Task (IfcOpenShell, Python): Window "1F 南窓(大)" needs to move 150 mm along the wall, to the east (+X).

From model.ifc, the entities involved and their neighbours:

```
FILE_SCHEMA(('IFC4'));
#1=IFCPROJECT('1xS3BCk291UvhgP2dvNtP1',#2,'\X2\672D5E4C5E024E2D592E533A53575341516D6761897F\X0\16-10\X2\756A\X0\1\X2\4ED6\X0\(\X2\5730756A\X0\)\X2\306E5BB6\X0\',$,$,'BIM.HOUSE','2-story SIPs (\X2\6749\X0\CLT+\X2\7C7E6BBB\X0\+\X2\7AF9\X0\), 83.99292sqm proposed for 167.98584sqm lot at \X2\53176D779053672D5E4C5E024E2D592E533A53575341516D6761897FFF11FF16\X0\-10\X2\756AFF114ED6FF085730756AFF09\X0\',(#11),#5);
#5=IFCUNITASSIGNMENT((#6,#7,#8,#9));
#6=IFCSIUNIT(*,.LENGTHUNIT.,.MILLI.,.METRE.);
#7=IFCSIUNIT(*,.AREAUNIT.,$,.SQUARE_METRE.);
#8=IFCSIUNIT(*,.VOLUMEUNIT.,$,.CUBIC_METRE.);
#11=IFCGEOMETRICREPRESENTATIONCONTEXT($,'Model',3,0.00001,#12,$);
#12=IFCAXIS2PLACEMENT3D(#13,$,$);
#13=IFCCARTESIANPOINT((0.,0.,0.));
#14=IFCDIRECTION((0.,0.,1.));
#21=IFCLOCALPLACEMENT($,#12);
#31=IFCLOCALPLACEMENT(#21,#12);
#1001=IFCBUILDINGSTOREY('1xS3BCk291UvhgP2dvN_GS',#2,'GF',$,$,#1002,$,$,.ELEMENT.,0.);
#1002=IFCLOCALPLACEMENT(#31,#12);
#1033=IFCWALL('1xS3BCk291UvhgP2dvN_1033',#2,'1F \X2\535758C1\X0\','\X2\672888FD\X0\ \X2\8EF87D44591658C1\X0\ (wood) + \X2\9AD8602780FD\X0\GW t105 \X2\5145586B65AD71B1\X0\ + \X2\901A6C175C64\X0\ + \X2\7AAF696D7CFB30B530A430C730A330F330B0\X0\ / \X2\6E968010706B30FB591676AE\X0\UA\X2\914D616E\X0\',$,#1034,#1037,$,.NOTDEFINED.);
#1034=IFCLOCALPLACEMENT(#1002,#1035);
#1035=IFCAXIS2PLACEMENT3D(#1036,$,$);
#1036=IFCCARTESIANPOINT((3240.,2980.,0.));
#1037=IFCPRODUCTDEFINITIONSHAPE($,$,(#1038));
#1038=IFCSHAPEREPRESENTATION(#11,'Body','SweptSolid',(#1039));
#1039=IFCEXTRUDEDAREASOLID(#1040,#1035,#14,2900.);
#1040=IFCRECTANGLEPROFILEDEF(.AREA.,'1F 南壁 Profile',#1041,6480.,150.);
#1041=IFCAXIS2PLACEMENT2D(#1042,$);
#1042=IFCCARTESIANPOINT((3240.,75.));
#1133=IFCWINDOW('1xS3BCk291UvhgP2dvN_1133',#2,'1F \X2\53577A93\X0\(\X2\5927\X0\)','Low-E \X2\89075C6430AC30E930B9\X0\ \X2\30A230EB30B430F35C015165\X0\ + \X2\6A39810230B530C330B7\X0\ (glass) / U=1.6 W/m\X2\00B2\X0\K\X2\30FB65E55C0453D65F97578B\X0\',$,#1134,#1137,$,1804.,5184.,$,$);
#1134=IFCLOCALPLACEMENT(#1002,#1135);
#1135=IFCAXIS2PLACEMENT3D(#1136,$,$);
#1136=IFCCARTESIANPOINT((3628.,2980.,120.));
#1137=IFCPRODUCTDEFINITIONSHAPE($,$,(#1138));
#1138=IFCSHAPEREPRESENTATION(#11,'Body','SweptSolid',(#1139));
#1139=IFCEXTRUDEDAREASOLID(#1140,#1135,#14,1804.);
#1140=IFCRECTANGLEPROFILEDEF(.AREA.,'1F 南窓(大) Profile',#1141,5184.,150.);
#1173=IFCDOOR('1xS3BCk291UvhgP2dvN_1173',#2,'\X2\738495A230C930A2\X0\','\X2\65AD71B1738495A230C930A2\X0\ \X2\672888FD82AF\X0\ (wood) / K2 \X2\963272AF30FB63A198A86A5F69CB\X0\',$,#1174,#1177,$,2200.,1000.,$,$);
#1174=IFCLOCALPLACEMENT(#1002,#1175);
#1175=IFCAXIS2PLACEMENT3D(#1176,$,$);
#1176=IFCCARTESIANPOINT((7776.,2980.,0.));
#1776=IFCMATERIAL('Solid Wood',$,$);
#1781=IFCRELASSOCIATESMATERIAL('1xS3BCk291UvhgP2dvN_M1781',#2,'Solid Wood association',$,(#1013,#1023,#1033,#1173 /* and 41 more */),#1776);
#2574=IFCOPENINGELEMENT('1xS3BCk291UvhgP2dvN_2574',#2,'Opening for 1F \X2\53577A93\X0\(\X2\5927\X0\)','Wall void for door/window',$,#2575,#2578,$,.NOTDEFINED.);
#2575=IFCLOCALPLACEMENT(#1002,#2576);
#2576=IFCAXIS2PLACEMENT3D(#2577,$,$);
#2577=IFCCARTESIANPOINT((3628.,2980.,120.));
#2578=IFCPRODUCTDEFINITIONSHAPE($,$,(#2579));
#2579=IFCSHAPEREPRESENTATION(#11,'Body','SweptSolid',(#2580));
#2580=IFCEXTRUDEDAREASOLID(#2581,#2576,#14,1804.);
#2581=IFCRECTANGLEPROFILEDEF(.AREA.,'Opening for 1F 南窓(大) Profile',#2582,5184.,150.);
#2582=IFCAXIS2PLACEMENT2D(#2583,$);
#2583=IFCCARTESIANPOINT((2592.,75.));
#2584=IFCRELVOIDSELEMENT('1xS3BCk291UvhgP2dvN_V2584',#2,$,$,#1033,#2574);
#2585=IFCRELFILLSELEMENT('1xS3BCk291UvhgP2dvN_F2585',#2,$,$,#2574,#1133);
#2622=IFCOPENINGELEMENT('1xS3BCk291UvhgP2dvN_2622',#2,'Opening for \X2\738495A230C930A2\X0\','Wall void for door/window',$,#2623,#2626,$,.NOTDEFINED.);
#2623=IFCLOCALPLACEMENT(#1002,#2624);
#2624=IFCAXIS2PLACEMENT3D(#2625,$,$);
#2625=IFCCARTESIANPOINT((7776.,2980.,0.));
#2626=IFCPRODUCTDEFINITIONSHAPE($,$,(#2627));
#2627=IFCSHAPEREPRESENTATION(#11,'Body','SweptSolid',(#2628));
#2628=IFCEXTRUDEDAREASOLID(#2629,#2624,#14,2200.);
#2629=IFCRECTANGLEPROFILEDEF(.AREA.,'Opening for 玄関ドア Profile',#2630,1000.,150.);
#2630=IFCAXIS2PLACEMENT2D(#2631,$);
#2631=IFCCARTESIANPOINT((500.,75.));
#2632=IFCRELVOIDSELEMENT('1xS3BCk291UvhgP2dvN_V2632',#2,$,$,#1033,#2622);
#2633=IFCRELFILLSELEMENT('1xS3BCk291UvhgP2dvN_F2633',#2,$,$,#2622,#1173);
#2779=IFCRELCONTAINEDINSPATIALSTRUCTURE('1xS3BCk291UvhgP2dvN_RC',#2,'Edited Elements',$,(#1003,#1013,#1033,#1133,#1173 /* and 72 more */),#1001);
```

```python
import ifcopenshell
import ifcopenshell.api.geometry
import ifcopenshell.util.placement
import ifcopenshell.util.unit

model = ifcopenshell.open("model.ifc")
unit_scale = ifcopenshell.util.unit.calculate_unit_scale(model)

window = model.by_id(1133)
opening = window.FillsVoids[0].RelatingOpeningElement
wall = opening.VoidsElements[0].RelatingBuildingElement

wall_matrix = ifcopenshell.util.placement.get_local_placement(wall.ObjectPlacement)
shift = wall_matrix[:3, 0] * 0.15 / unit_scale
before = ifcopenshell.util.placement.get_local_placement(window.ObjectPlacement)[:3, 3].copy()

# The window is not placed relative to its opening, so move both.
for product in (opening, window):
    matrix = ifcopenshell.util.placement.get_local_placement(product.ObjectPlacement)
    matrix[:3, 3] += shift
    ifcopenshell.api.geometry.edit_object_placement(model, product=product, matrix=matrix, is_si=False)

after = ifcopenshell.util.placement.get_local_placement(window.ObjectPlacement)[:3, 3]
print("window moved by", (after - before).round(3) + 0.0)

model.write("model_updated.ifc")
```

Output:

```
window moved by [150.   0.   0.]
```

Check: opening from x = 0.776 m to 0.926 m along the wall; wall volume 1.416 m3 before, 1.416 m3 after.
